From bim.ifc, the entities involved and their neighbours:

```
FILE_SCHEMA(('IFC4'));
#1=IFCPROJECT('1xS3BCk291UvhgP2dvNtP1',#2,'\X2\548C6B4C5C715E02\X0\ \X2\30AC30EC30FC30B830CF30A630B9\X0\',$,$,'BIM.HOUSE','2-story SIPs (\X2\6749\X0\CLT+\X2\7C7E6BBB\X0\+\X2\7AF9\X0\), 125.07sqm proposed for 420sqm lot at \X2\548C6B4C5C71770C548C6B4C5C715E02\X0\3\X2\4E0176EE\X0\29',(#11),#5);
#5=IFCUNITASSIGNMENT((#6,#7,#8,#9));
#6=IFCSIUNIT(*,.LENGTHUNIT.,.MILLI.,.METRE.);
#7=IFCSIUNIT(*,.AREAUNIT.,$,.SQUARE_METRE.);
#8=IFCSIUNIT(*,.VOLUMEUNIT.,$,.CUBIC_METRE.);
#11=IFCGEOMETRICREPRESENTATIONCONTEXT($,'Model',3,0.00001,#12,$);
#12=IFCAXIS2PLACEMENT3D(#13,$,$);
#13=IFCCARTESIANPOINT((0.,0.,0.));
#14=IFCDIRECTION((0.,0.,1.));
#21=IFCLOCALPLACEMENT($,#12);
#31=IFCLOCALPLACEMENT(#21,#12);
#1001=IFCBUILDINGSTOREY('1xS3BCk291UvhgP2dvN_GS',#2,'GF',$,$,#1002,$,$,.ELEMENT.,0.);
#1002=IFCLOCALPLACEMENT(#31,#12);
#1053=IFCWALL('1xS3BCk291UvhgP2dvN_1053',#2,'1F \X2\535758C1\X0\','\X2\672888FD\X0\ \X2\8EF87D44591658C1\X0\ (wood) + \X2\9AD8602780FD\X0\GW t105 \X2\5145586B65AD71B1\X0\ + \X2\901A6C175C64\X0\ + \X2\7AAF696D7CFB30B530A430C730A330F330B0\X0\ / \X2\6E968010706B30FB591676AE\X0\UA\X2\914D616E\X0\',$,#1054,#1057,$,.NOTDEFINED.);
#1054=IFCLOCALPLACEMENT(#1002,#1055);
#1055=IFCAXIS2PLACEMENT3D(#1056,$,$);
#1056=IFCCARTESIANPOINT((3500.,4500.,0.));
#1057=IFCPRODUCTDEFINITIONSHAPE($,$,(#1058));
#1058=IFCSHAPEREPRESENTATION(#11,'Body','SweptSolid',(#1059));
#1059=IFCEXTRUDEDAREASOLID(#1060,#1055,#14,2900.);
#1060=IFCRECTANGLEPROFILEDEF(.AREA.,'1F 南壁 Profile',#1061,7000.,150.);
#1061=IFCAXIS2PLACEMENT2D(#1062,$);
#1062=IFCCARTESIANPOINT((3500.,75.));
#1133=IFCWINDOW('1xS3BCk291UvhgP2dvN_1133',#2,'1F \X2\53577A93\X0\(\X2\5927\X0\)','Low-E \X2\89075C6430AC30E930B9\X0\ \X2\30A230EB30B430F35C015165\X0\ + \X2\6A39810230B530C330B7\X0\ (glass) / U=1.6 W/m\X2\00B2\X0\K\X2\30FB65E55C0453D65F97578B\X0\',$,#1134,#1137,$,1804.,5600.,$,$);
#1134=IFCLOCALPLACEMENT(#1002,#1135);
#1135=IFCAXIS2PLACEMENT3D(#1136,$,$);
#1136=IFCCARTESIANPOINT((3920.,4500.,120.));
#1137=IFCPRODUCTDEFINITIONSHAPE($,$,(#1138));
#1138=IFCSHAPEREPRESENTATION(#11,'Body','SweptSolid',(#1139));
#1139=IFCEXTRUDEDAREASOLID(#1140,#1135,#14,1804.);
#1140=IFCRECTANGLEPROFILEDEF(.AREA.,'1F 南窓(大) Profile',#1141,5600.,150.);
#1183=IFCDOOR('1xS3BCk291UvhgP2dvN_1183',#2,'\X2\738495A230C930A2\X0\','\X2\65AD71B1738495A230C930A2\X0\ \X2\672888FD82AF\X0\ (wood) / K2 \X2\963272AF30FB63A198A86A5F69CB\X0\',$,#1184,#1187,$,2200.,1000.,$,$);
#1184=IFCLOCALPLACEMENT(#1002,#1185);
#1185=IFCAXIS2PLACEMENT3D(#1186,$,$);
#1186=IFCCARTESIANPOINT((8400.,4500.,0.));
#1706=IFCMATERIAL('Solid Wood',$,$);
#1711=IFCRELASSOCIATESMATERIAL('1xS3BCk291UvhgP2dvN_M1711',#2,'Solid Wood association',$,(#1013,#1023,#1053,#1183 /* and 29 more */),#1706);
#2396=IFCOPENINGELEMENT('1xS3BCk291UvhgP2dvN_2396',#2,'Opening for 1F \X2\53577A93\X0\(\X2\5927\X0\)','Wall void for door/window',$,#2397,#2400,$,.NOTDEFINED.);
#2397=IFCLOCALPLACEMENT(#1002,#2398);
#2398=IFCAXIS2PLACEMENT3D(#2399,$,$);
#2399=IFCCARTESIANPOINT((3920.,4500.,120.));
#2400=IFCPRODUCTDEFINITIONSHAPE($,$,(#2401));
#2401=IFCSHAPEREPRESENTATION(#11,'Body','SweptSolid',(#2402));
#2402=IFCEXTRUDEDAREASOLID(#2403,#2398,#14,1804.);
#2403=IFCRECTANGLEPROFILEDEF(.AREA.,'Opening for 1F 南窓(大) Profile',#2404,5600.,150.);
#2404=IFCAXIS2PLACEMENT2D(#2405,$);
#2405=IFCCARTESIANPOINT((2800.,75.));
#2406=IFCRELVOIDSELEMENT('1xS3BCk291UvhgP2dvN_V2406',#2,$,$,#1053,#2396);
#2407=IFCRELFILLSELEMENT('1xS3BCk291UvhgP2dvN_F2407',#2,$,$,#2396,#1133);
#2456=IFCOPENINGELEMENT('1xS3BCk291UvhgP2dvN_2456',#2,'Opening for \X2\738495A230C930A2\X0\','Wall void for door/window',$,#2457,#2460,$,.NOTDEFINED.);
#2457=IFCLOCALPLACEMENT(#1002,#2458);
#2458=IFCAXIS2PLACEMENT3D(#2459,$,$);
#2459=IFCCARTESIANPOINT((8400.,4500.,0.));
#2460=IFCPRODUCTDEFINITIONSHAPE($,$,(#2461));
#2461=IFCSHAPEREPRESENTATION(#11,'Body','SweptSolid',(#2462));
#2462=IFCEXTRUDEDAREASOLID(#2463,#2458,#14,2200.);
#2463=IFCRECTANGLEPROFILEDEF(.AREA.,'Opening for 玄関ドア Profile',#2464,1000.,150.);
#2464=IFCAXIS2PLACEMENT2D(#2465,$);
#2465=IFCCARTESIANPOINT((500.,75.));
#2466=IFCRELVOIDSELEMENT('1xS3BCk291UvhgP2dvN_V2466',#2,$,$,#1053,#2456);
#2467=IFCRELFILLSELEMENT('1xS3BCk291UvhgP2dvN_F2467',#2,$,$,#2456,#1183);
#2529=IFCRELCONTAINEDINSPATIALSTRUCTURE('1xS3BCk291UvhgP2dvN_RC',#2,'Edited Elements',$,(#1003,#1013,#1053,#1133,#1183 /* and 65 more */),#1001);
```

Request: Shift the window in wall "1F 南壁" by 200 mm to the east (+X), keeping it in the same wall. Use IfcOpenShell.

```python
import ifcopenshell
import ifcopenshell.api.geometry
import ifcopenshell.util.placement
import ifcopenshell.util.unit

model = ifcopenshell.open("bim.ifc")
unit_scale = ifcopenshell.util.unit.calculate_unit_scale(model)

window = model.by_guid("1xS3BCk291UvhgP2dvN_1133")
opening = window.FillsVoids[0].RelatingOpeningElement
wall = opening.VoidsElements[0].RelatingBuildingElement

wall_matrix = ifcopenshell.util.placement.get_local_placement(wall.ObjectPlacement)
shift = wall_matrix[:3, 0] * 0.2 / unit_scale
before = ifcopenshell.util.placement.get_local_placement(window.ObjectPlacement)[:3, 3].copy()

# The window is not placed relative to its opening, so move both.
for product in (opening, window):
    matrix = ifcopenshell.util.placement.get_local_placement(product.ObjectPlacement)
    matrix[:3, 3] += shift
    ifcopenshell.api.geometry.edit_object_placement(model, product=product, matrix=matrix, is_si=False)

after = ifcopenshell.util.placement.get_local_placement(window.ObjectPlacement)[:3, 3]
print("window moved by", (after - before).round(3) + 0.0)

model.write("bim_edited.ifc")
```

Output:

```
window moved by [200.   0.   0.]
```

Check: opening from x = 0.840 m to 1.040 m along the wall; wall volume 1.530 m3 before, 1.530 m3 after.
